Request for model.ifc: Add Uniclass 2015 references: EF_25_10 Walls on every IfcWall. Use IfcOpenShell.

First a look at what the model holds.

```python
import ifcopenshell

model = ifcopenshell.open("model.ifc")
print(model.schema)
print("classifications:", [c.Name for c in model.by_type("IfcClassification")])
for ifc_class in ("IfcDoor", "IfcRoof", "IfcStair", "IfcWall", "IfcWindow"):
    print(ifc_class, len(model.by_type(ifc_class)))
```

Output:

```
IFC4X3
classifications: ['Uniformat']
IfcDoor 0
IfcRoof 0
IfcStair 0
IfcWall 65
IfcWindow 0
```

```python
import ifcopenshell
import ifcopenshell.api.classification

model = ifcopenshell.open("model.ifc")

system = ifcopenshell.api.classification.add_classification(model, classification="Uniclass 2015")

codes = {
    "IfcWall": ("EF_25_10", "Walls"),
}
for ifc_class, (code, name) in codes.items():
    products = model.by_type(ifc_class)
    ifcopenshell.api.classification.add_reference(
        model, products=products, classification=system, identification=code, name=name
    )
    print(code, len(products))

model.write("model_rev.ifc")
```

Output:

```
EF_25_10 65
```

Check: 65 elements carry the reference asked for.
